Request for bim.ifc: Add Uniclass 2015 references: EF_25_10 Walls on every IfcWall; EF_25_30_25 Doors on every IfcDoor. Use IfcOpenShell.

First a look at what the model holds.

```python
import ifcopenshell

model = ifcopenshell.open("bim.ifc")
print(model.schema)
print("classifications:", [c.Name for c in model.by_type("IfcClassification")])
for ifc_class in ("IfcDoor", "IfcRoof", "IfcStair", "IfcWall", "IfcWindow"):
    print(ifc_class, len(model.by_type(ifc_class)))
```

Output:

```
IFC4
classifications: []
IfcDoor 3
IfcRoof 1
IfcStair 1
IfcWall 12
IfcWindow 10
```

```python
import ifcopenshell
import ifcopenshell.api.classification

model = ifcopenshell.open("bim.ifc")

system = ifcopenshell.api.classification.add_classification(model, classification="Uniclass 2015")

codes = {
    "IfcWall": ("EF_25_10", "Walls"),
    "IfcDoor": ("EF_25_30_25", "Doors"),
}
for ifc_class, (code, name) in codes.items():
    products = model.by_type(ifc_class)
    ifcopenshell.api.classification.add_reference(
        model, products=products, classification=system, identification=code, name=name
    )
    print(code, len(products))

model.write("bim_edited.ifc")
```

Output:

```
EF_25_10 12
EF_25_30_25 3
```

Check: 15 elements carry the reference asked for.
